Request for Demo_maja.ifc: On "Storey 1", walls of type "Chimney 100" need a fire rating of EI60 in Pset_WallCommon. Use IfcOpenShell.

First a look at what the model holds.

```python
import ifcopenshell
import ifcopenshell.util.element

model = ifcopenshell.open("Demo_maja.ifc")
print(model.schema)
storey = next(s for s in model.by_type("IfcBuildingStorey") if s.Name == "Storey 1")
walls = [e for e in ifcopenshell.util.element.get_decomposition(storey) if e.is_a("IfcWall")]
seen = {}
for e in walls:
    element_type = ifcopenshell.util.element.get_type(e)
    key = (element_type.Name if element_type != e and element_type else None, ifcopenshell.util.element.get_pset(e, "Pset_WallCommon", "FireRating"))
    seen[key] = seen.get(key, 0) + 1
for (name, value), count in sorted(seen.items(), key=str):
    print(count, "x", name, "|", value)
```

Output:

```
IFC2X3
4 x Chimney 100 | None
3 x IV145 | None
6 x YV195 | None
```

```python
import ifcopenshell
import ifcopenshell.api.pset
import ifcopenshell.util.element

model = ifcopenshell.open("Demo_maja.ifc")

storey = next(s for s in model.by_type("IfcBuildingStorey") if s.Name == "Storey 1")
walls = [e for e in ifcopenshell.util.element.get_decomposition(storey) if e.is_a("IfcWall")]

count = 0
for e in walls:
    element_type = ifcopenshell.util.element.get_type(e)
    if element_type in (None, e) or element_type.Name != "Chimney 100":
        continue
    # add_pset returns the element's existing set when there is one.
    pset = ifcopenshell.api.pset.add_pset(model, product=e, name="Pset_WallCommon")
    ifcopenshell.api.pset.edit_pset(model, pset=pset, properties={"FireRating": "EI60"})
    count += 1

print(count, "walls updated")

model.write("Demo_maja_edited.ifc")
```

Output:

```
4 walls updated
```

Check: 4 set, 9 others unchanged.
